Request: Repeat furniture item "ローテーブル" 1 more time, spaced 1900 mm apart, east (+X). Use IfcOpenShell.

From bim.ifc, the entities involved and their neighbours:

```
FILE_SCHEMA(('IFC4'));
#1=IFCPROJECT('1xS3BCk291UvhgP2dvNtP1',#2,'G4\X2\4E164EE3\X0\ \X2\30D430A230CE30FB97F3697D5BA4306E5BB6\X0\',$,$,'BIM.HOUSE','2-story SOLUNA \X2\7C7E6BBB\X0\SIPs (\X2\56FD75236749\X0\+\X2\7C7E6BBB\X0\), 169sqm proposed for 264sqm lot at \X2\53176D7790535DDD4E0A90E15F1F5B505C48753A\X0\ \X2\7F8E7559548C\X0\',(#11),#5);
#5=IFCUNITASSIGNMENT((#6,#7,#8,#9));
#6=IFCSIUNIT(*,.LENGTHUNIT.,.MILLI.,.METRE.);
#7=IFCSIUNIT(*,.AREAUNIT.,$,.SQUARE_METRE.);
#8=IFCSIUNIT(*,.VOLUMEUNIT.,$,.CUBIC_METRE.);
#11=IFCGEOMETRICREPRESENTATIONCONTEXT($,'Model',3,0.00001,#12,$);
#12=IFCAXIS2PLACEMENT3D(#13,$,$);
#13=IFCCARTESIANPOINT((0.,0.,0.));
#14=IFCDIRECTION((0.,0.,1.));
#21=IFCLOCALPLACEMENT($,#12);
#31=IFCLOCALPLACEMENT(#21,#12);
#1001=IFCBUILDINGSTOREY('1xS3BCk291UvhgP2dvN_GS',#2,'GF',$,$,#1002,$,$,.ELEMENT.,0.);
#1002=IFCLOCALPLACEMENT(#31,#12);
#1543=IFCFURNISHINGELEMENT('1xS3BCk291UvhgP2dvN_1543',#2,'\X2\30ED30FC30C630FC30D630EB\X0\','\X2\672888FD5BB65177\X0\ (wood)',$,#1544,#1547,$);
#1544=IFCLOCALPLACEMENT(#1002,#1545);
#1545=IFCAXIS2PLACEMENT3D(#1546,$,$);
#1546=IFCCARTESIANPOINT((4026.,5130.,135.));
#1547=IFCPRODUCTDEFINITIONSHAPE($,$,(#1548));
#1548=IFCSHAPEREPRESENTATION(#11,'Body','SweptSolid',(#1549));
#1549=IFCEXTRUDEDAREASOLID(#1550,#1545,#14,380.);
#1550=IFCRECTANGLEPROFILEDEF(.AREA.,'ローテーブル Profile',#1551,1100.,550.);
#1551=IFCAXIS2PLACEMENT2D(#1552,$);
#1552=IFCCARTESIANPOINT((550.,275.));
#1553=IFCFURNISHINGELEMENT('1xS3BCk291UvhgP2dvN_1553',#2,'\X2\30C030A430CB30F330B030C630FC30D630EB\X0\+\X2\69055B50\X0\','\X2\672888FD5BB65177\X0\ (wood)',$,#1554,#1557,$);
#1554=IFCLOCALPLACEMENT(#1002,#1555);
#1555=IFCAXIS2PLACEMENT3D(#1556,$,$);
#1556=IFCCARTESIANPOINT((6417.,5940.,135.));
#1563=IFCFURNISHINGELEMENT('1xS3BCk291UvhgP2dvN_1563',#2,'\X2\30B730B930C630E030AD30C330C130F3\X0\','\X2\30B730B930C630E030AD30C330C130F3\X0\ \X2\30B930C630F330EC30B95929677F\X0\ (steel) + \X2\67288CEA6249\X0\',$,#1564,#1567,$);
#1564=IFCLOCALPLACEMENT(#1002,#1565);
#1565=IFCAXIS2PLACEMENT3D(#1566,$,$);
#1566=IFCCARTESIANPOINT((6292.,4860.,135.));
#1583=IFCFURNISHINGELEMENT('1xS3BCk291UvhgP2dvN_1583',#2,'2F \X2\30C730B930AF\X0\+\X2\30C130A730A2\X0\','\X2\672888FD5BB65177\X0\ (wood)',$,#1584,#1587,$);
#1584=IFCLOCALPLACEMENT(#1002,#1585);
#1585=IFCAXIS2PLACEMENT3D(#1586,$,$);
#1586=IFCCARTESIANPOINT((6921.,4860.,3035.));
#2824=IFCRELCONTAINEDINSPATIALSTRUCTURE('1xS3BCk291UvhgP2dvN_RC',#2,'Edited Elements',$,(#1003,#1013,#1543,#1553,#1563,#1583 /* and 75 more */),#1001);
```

```python
import numpy as np
import ifcopenshell
import ifcopenshell.api.geometry
import ifcopenshell.api.root
import ifcopenshell.util.element
import ifcopenshell.util.placement

model = ifcopenshell.open("bim.ifc")


def reuse_history(source, copy):
    """copy_class also copies each property set's owner history, people and application; keep the originals."""
    for rel in copy.IsDefinedBy:
        if rel.is_a("IfcRelDefinesByProperties") and (history := rel.RelatingPropertyDefinition.OwnerHistory):
            rel.RelatingPropertyDefinition.OwnerHistory = source.OwnerHistory
            ifcopenshell.util.element.remove_deep2(model, history)


source = model.by_guid("1xS3BCk291UvhgP2dvN_1543")
base = ifcopenshell.util.placement.get_local_placement(source.ObjectPlacement)
step = np.array([1.0, 0.0, 0.0]) * 1900.0

for i in range(1, 2):
    copy = ifcopenshell.api.root.copy_class(model, product=source)
    copy.Representation = ifcopenshell.util.element.copy_deep(
        model, source.Representation, exclude=["IfcGeometricRepresentationContext", "IfcRepresentationMap"]
    )
    reuse_history(source, copy)
    matrix = base.copy()
    matrix[:3, 3] += i * step
    print("added at", matrix[:3, 3].round(3) + 0.0)
    ifcopenshell.api.geometry.edit_object_placement(model, product=copy, matrix=matrix, is_si=False)

model.write("bim_updated.ifc")
```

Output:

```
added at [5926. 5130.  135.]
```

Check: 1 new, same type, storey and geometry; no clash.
